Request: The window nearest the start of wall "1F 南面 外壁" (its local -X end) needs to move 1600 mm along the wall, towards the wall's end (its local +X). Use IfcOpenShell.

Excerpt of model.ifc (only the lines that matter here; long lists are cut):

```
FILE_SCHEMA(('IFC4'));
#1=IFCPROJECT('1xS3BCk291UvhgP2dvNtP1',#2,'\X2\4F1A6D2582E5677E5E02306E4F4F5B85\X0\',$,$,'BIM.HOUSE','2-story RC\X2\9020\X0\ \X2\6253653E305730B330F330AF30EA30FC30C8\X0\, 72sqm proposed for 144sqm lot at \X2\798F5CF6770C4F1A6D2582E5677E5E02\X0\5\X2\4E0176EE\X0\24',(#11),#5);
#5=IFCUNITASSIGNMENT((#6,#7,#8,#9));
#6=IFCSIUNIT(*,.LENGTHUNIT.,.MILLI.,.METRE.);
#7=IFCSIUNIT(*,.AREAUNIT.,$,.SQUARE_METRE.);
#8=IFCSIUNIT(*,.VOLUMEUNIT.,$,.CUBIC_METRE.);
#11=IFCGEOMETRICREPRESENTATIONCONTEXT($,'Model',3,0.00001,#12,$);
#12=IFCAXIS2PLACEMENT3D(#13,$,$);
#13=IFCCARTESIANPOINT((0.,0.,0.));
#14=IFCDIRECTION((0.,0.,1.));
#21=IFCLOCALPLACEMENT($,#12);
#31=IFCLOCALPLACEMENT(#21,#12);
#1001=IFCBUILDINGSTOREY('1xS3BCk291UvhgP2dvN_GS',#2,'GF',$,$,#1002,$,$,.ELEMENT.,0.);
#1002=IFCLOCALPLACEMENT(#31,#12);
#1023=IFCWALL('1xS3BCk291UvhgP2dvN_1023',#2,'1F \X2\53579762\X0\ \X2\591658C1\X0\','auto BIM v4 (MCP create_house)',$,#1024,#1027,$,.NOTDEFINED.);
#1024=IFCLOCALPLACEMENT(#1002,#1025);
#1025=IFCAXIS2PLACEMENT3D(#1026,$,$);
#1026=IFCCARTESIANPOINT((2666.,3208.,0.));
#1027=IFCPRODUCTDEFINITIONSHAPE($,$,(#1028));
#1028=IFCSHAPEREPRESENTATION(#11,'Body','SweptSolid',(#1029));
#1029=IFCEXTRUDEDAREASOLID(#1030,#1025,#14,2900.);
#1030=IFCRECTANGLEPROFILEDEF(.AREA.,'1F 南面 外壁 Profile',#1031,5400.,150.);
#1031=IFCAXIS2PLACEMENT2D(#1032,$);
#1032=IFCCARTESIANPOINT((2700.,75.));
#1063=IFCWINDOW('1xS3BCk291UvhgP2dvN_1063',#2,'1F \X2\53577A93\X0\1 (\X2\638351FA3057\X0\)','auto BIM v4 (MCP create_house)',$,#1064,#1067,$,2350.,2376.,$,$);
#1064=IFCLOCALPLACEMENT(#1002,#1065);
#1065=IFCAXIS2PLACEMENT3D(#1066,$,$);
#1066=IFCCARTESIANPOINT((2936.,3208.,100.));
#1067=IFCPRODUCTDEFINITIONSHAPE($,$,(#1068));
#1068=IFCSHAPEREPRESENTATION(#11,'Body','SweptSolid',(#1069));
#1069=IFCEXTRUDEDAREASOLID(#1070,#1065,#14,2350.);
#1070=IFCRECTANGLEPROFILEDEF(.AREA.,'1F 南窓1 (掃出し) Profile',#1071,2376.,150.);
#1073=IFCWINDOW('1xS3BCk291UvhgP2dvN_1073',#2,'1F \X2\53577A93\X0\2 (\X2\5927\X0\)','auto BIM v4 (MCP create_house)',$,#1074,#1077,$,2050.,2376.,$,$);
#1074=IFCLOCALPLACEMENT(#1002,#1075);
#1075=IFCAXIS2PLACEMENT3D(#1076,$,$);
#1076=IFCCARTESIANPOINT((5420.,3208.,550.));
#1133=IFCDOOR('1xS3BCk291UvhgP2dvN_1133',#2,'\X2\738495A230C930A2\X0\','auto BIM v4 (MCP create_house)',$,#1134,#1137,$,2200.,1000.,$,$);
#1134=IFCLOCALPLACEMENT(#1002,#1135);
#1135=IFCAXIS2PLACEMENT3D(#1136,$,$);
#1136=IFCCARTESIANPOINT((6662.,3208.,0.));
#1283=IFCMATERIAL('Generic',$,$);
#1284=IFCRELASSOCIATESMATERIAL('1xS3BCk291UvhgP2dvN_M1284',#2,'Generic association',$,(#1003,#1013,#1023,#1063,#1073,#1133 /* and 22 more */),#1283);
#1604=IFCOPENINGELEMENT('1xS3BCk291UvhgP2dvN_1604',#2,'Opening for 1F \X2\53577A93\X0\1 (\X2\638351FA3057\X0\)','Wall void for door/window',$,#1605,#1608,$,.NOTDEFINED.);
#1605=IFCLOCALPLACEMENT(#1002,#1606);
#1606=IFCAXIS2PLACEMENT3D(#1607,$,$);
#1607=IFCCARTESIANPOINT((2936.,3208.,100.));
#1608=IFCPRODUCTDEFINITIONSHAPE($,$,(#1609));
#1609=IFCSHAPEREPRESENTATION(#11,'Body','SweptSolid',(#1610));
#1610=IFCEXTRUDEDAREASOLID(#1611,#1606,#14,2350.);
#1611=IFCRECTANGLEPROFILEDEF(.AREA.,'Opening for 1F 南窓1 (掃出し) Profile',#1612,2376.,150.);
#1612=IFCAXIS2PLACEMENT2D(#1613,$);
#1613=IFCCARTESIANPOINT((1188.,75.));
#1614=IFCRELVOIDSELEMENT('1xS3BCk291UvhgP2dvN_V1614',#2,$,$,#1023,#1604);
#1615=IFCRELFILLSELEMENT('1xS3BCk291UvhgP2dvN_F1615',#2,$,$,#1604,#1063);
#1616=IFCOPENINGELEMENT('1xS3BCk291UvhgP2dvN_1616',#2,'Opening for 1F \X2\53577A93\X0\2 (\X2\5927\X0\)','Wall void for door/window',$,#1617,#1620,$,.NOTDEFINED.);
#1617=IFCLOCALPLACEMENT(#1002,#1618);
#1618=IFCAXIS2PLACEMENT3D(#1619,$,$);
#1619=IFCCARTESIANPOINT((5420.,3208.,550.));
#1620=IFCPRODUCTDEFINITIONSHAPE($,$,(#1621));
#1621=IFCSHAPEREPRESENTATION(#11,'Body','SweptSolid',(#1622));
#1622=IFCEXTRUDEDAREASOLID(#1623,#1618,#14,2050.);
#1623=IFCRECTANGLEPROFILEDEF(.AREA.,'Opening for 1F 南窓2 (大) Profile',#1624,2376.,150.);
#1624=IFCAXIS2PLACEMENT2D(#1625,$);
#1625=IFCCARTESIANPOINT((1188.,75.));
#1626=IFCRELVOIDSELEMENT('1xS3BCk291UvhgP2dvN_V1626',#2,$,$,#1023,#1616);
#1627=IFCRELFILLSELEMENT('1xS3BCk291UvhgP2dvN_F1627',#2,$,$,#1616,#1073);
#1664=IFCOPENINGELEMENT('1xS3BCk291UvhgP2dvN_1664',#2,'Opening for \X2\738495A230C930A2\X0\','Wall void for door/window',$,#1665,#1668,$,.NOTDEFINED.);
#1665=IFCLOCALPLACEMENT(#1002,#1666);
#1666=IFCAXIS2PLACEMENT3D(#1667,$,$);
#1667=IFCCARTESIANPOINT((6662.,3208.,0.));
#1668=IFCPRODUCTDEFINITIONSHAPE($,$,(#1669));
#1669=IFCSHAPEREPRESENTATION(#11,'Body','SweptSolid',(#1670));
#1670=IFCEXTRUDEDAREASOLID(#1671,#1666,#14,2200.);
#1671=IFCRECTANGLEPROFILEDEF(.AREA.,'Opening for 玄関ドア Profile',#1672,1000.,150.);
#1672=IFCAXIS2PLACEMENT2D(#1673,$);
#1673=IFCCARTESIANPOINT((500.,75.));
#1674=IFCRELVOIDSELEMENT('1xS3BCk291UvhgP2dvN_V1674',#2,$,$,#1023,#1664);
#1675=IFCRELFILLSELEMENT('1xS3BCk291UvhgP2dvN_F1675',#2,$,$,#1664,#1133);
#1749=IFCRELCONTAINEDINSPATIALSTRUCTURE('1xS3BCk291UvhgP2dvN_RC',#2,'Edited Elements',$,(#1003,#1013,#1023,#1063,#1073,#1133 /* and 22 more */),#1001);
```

```python
import ifcopenshell
import ifcopenshell.api.geometry
import ifcopenshell.util.placement
import ifcopenshell.util.unit

model = ifcopenshell.open("model.ifc")
unit_scale = ifcopenshell.util.unit.calculate_unit_scale(model)

window = model.by_guid("1xS3BCk291UvhgP2dvN_1063")
opening = window.FillsVoids[0].RelatingOpeningElement
wall = opening.VoidsElements[0].RelatingBuildingElement

wall_matrix = ifcopenshell.util.placement.get_local_placement(wall.ObjectPlacement)
shift = wall_matrix[:3, 0] * 1.6 / unit_scale
before = ifcopenshell.util.placement.get_local_placement(window.ObjectPlacement)[:3, 3].copy()

# The window is not placed relative to its opening, so move both.
for product in (opening, window):
    matrix = ifcopenshell.util.placement.get_local_placement(product.ObjectPlacement)
    matrix[:3, 3] += shift
    ifcopenshell.api.geometry.edit_object_placement(model, product=product, matrix=matrix, is_si=False)

after = ifcopenshell.util.placement.get_local_placement(window.ObjectPlacement)[:3, 3]
print("window moved by", (after - before).round(3) + 0.0)

model.write("model-out.ifc")
```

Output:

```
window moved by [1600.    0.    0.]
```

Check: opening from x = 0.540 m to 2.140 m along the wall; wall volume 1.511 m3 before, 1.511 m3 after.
